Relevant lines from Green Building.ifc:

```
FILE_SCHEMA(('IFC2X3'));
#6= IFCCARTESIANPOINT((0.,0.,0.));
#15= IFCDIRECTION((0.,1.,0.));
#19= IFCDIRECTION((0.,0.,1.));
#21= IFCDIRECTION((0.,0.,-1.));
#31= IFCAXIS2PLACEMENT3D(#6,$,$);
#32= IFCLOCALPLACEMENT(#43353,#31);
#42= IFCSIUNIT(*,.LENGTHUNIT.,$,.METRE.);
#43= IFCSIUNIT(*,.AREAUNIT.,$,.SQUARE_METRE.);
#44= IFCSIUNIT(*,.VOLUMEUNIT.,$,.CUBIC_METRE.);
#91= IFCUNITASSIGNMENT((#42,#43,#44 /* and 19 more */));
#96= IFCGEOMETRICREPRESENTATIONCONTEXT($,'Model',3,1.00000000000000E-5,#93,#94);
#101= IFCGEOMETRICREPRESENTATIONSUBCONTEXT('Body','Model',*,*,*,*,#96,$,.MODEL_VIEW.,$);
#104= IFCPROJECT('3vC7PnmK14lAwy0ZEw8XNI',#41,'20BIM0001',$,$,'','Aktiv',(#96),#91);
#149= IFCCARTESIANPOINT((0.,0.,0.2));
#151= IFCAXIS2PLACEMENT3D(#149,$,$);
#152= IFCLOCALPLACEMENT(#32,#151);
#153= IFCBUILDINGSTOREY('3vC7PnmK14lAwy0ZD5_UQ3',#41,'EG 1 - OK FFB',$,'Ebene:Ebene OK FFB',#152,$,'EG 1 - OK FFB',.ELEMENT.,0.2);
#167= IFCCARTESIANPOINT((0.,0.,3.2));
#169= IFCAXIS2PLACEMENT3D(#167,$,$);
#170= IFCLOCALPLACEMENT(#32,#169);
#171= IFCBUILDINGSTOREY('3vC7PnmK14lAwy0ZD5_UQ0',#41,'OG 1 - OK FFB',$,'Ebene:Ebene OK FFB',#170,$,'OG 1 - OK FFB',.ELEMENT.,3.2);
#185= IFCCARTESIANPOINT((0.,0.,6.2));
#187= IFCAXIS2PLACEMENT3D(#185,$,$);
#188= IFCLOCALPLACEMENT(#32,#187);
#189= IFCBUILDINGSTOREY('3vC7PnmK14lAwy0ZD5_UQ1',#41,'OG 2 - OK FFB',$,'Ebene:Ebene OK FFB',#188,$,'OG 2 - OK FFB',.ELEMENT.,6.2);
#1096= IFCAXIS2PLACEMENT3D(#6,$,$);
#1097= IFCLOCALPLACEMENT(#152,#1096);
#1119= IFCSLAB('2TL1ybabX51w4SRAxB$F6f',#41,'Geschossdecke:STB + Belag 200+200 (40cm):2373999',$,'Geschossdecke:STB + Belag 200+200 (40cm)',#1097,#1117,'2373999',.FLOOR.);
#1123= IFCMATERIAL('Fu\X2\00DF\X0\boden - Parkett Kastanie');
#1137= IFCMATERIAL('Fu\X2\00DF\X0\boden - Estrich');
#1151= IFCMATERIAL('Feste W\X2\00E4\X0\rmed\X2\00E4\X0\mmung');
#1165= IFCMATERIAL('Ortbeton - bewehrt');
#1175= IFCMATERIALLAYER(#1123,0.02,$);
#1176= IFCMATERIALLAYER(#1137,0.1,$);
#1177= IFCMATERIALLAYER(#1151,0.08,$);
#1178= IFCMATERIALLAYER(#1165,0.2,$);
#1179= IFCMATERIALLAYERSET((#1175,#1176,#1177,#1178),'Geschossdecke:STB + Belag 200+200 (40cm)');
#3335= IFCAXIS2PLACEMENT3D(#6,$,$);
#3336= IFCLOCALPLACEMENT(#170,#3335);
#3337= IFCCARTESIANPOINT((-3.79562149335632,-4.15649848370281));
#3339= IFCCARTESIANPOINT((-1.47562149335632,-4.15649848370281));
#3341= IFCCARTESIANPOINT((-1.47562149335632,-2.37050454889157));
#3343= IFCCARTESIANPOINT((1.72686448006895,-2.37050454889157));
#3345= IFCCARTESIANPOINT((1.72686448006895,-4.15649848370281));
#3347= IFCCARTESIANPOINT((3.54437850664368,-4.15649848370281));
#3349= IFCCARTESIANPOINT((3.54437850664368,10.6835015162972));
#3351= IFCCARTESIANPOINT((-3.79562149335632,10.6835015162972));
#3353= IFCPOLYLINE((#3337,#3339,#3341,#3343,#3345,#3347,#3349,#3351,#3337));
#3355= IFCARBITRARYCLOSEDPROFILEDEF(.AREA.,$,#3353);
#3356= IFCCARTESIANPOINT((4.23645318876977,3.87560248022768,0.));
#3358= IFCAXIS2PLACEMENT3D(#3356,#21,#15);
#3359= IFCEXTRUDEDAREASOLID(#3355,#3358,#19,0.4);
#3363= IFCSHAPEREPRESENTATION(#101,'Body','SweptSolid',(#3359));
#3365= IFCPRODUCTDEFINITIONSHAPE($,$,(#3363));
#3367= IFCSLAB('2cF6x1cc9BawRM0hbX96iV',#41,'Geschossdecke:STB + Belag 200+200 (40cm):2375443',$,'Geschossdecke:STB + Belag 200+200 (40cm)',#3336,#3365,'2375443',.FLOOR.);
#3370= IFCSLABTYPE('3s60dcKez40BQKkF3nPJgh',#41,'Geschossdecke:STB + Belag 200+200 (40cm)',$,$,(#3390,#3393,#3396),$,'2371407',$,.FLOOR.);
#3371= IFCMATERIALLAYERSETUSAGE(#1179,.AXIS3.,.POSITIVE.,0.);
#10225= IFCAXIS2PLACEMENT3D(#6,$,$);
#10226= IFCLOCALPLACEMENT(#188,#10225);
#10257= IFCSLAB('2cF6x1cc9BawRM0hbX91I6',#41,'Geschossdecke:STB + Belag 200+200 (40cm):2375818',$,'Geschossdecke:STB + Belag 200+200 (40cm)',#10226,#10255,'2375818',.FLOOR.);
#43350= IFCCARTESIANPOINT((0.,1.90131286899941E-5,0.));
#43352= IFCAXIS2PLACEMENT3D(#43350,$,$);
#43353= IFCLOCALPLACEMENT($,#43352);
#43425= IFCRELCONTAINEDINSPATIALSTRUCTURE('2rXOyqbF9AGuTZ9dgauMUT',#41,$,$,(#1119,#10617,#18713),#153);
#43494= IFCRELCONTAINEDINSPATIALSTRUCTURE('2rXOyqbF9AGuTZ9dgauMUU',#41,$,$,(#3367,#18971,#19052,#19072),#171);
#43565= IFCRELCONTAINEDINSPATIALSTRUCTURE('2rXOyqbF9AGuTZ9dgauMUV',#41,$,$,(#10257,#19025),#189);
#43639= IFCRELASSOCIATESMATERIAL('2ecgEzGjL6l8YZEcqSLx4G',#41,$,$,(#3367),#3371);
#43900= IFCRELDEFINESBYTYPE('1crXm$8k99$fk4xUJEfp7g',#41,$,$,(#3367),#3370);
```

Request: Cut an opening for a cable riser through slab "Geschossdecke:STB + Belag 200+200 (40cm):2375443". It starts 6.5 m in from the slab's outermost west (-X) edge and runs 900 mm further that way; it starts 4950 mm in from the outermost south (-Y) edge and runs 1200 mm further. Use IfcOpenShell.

```python
import numpy as np
import ifcopenshell
import ifcopenshell.api.feature
import ifcopenshell.api.geometry
import ifcopenshell.api.root
import ifcopenshell.geom
import ifcopenshell.util.placement
import ifcopenshell.util.representation
import ifcopenshell.util.shape
import ifcopenshell.util.unit

model = ifcopenshell.open("Green Building.ifc")
unit_scale = ifcopenshell.util.unit.calculate_unit_scale(model)
settings = ifcopenshell.geom.settings()


def volume(element):
    """Net volume in cubic metres, openings subtracted."""
    shape = ifcopenshell.geom.create_shape(settings, element)
    return ifcopenshell.util.shape.get_volume(shape.geometry)


slab = model.by_guid("2cF6x1cc9BawRM0hbX96iV")
before = volume(slab)

# Extent in the slab's own axes, in metres. The edges named are its -X and -Y sides.
slab_shape = ifcopenshell.geom.create_shape(settings, slab)
vertices = ifcopenshell.util.shape.get_vertices(slab_shape.geometry)
x_min, y_min, bottom = vertices.min(axis=0)
top = vertices[:, 2].max()

opening = ifcopenshell.api.root.create_entity(model, ifc_class="IfcOpeningElement", name="Cable riser opening")
context = ifcopenshell.util.representation.get_context(model, "Model", "Body", "MODEL_VIEW")
width, depth = 0.9, 1.2
outline = [(0.0, 0.0), (width, 0.0), (width, depth), (0.0, depth), (0.0, 0.0)]
# Overshoot both faces by 50 mm so the cut is clean.
shape = ifcopenshell.api.geometry.add_slab_representation(
    model, context=context, depth=top - bottom + 0.1, polyline=outline
)
ifcopenshell.api.geometry.assign_representation(model, product=opening, representation=shape)

matrix = ifcopenshell.util.placement.get_local_placement(slab.ObjectPlacement)
matrix[:, 3] = matrix @ np.append(np.array([x_min + 6.5, y_min + 4.95, bottom - 0.05]) / unit_scale, 1.0)
ifcopenshell.api.geometry.edit_object_placement(model, product=opening, matrix=matrix, is_si=False)
ifcopenshell.api.feature.add_feature(model, feature=opening, element=slab)

after = volume(slab)

print(f"slab volume {before:.3f} -> {after:.3f} m3")

model.write("Green Building_updated.ifc")
```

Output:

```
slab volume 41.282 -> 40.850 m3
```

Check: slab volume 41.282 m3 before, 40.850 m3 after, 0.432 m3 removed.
